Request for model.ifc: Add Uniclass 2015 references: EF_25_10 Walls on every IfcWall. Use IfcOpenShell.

First a look at what the model holds.

```python
import ifcopenshell

model = ifcopenshell.open("model.ifc")
print(model.schema)
print("classifications:", [c.Name for c in model.by_type("IfcClassification")])
for ifc_class in ("IfcDoor", "IfcRoof", "IfcStair", "IfcWall", "IfcWindow"):
    print(ifc_class, len(model.by_type(ifc_class)))
```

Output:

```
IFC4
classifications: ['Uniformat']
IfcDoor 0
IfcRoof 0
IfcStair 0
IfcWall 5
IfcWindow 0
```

```python
import ifcopenshell
import ifcopenshell.api.classification

model = ifcopenshell.open("model.ifc")

system = ifcopenshell.api.classification.add_classification(model, classification="Uniclass 2015")

codes = {
    "IfcWall": ("EF_25_10", "Walls"),
}
for ifc_class, (code, name) in codes.items():
    products = model.by_type(ifc_class)
    ifcopenshell.api.classification.add_reference(
        model, products=products, classification=system, identification=code, name=name
    )
    print(code, len(products))

model.write("model_edited.ifc")
```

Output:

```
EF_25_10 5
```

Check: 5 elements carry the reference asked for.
